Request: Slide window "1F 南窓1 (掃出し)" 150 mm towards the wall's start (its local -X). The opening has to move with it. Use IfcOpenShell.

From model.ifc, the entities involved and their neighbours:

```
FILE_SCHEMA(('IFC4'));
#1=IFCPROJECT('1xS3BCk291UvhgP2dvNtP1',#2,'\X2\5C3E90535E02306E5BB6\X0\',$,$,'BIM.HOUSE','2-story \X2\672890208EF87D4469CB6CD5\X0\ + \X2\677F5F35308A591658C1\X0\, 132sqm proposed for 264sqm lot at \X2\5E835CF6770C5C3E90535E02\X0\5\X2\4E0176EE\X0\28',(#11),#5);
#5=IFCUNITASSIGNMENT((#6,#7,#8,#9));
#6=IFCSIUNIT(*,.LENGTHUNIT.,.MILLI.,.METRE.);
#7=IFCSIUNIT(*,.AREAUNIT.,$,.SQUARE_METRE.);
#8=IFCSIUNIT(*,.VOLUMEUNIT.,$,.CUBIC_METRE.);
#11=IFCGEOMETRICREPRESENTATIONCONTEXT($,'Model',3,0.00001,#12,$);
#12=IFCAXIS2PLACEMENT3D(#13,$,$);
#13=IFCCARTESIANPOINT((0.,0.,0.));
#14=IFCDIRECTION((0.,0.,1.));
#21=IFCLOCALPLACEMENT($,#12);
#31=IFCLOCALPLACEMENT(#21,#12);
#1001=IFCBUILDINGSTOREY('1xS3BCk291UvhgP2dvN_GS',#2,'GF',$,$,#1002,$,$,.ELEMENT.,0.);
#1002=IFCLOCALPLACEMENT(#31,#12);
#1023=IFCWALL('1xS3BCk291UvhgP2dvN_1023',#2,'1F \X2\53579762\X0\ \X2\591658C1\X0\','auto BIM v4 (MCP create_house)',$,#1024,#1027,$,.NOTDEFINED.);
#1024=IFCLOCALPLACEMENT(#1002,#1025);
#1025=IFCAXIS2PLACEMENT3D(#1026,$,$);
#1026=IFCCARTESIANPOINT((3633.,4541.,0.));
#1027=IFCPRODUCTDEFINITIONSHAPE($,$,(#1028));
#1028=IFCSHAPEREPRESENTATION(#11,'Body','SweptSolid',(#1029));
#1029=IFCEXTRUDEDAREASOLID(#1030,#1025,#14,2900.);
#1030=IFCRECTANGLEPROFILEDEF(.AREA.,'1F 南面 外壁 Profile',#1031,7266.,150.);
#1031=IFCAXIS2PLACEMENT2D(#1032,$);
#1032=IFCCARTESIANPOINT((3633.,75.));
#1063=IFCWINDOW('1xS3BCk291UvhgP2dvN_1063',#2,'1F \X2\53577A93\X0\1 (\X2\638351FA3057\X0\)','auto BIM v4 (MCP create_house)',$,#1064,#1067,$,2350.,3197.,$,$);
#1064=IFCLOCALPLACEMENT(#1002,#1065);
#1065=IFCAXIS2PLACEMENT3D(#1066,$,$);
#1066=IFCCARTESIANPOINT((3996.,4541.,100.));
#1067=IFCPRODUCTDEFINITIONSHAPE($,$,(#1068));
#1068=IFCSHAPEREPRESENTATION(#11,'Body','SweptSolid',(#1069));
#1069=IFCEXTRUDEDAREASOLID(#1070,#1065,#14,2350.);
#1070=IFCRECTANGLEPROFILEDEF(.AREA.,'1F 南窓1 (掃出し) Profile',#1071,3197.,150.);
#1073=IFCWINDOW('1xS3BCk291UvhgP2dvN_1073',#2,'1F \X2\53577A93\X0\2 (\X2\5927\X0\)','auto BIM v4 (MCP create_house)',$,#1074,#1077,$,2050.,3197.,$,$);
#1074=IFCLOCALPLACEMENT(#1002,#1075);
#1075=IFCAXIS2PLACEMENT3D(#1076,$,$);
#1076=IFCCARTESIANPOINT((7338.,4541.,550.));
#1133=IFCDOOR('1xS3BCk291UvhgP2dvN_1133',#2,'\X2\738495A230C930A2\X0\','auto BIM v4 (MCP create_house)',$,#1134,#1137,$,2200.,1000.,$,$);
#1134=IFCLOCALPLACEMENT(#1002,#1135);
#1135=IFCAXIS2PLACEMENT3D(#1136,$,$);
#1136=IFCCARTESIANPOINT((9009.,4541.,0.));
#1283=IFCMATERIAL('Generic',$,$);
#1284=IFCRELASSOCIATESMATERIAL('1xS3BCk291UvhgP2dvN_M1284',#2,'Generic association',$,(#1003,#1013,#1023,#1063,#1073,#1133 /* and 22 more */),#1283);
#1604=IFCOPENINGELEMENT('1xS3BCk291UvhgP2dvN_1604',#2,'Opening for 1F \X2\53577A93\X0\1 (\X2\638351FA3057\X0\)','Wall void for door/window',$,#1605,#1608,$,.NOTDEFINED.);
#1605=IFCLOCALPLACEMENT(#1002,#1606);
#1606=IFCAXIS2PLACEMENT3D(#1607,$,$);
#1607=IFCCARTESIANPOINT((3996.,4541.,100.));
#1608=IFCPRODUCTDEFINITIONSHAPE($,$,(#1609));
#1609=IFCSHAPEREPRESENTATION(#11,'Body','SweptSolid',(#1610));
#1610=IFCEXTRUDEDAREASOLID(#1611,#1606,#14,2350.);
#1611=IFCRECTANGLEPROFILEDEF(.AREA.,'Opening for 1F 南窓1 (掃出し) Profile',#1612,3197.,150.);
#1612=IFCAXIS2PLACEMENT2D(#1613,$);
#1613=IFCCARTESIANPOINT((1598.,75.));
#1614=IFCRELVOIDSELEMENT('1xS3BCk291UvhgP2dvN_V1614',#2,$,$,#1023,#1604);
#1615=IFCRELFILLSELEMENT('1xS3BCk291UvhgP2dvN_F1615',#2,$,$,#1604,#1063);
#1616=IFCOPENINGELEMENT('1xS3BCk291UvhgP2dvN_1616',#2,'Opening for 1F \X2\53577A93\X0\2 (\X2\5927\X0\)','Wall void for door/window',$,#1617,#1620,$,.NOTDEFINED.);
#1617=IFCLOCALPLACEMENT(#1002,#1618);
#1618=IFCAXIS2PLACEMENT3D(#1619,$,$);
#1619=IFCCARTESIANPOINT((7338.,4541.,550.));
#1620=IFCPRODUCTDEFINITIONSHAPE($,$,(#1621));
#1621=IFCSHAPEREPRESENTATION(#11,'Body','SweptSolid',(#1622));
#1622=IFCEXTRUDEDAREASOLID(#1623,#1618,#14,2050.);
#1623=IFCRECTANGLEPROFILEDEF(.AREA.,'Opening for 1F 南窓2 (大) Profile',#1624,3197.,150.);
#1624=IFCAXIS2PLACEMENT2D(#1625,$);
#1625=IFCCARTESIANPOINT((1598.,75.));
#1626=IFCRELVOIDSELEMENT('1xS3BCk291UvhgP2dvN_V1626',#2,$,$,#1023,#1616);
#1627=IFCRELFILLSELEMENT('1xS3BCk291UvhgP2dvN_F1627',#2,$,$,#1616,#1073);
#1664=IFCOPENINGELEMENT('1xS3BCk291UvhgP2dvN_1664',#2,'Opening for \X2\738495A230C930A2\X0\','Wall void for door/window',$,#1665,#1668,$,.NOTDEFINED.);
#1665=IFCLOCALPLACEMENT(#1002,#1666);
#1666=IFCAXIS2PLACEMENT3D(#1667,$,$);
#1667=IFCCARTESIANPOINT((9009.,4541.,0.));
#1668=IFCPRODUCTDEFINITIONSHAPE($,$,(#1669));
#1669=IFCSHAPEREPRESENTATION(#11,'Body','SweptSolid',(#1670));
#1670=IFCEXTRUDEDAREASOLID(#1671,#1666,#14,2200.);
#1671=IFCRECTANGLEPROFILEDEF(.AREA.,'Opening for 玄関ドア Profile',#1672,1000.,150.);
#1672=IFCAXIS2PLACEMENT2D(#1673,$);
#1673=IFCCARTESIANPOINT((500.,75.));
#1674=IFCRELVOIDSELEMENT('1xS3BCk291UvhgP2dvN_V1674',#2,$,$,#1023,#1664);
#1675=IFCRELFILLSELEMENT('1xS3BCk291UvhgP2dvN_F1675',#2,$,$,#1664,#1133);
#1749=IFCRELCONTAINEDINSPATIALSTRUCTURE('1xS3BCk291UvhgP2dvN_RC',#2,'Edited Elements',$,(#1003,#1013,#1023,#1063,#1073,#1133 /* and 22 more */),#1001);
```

```python
import ifcopenshell
import ifcopenshell.api.geometry
import ifcopenshell.util.placement

model = ifcopenshell.open("model.ifc")

window = model.by_guid("1xS3BCk291UvhgP2dvN_1063")
opening = window.FillsVoids[0].RelatingOpeningElement
wall = opening.VoidsElements[0].RelatingBuildingElement

wall_matrix = ifcopenshell.util.placement.get_local_placement(wall.ObjectPlacement)
shift = wall_matrix[:3, 0] * -150.0
before = ifcopenshell.util.placement.get_local_placement(window.ObjectPlacement)[:3, 3].copy()

# The window is not placed relative to its opening, so move both.
for product in (opening, window):
    matrix = ifcopenshell.util.placement.get_local_placement(product.ObjectPlacement)
    matrix[:3, 3] += shift
    ifcopenshell.api.geometry.edit_object_placement(model, product=product, matrix=matrix, is_si=False)

after = ifcopenshell.util.placement.get_local_placement(window.ObjectPlacement)[:3, 3]
print("window moved by", (after - before).round(3) + 0.0)

model.write("model-out.ifc")
```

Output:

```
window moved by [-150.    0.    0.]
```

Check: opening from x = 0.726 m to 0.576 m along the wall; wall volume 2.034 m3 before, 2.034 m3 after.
